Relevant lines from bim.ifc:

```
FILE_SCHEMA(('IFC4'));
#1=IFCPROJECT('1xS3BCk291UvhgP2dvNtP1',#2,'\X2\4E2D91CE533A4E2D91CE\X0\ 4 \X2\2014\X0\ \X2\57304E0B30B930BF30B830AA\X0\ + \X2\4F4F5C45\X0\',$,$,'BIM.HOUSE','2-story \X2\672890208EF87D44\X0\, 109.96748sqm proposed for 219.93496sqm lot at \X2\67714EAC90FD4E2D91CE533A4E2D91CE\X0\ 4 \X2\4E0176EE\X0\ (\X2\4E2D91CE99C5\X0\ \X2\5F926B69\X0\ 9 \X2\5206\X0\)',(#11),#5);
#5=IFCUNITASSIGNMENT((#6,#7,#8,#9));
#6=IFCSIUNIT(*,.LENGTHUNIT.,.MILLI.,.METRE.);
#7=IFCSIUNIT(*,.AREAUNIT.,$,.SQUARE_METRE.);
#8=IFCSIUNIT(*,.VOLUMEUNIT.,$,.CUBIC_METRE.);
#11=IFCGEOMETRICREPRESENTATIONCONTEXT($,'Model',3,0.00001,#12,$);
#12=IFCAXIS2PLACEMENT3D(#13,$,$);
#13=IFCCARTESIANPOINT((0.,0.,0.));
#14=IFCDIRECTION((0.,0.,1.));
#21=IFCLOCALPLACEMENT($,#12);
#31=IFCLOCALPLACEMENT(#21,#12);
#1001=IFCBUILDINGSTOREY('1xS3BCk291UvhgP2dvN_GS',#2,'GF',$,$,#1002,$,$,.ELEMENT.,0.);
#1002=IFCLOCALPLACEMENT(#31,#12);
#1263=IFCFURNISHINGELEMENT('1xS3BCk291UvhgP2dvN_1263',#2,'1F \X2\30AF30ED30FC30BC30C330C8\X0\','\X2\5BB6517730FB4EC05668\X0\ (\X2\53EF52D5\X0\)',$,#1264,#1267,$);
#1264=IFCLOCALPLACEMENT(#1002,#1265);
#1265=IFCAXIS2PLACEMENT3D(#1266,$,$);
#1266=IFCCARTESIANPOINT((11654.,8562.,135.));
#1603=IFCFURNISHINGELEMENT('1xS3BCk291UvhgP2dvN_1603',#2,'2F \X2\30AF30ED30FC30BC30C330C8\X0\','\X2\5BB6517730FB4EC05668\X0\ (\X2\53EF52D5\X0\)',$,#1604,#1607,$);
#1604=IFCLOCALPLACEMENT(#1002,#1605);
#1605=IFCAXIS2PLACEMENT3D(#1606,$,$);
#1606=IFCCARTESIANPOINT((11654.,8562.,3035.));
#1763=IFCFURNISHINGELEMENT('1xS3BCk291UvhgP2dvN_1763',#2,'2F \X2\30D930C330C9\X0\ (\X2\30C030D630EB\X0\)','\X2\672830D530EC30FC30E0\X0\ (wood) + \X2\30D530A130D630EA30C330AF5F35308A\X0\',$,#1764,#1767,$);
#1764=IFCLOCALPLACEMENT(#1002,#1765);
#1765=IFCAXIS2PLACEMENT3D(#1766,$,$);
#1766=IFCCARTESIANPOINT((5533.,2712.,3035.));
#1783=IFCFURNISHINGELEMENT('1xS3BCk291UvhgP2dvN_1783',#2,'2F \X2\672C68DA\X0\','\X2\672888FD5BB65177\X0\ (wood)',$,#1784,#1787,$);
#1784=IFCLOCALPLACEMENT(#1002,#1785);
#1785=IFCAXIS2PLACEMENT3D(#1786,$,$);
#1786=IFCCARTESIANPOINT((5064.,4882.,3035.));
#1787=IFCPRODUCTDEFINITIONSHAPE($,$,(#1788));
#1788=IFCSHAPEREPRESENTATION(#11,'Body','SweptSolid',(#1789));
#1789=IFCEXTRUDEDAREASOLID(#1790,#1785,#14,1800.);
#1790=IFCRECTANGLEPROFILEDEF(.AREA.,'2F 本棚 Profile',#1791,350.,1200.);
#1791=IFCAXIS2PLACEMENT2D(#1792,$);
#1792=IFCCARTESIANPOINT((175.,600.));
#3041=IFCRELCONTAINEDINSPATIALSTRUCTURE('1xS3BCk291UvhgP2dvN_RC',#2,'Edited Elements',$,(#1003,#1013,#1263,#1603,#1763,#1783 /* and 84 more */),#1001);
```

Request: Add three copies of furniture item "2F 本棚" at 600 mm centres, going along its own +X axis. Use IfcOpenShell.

```python
import ifcopenshell
import ifcopenshell.api.geometry
import ifcopenshell.api.root
import ifcopenshell.util.element
import ifcopenshell.util.placement
import ifcopenshell.util.unit

model = ifcopenshell.open("bim.ifc")
unit_scale = ifcopenshell.util.unit.calculate_unit_scale(model)


def reuse_history(source, copy):
    """copy_class also copies each property set's owner history, people and application; keep the originals."""
    for rel in copy.IsDefinedBy:
        if rel.is_a("IfcRelDefinesByProperties") and (history := rel.RelatingPropertyDefinition.OwnerHistory):
            rel.RelatingPropertyDefinition.OwnerHistory = source.OwnerHistory
            ifcopenshell.util.element.remove_deep2(model, history)


source = model.by_guid("1xS3BCk291UvhgP2dvN_1783")
base = ifcopenshell.util.placement.get_local_placement(source.ObjectPlacement)
step = base[:3, 0] * 0.6 / unit_scale

for i in range(1, 4):
    copy = ifcopenshell.api.root.copy_class(model, product=source)
    copy.Representation = ifcopenshell.util.element.copy_deep(
        model, source.Representation, exclude=["IfcGeometricRepresentationContext", "IfcRepresentationMap"]
    )
    reuse_history(source, copy)
    matrix = base.copy()
    matrix[:3, 3] += i * step
    print("added at", matrix[:3, 3].round(3) + 0.0)
    ifcopenshell.api.geometry.edit_object_placement(model, product=copy, matrix=matrix, is_si=False)

model.write("bim_v2.ifc")
```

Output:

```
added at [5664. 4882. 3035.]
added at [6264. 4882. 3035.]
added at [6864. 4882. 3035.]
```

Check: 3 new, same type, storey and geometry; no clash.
